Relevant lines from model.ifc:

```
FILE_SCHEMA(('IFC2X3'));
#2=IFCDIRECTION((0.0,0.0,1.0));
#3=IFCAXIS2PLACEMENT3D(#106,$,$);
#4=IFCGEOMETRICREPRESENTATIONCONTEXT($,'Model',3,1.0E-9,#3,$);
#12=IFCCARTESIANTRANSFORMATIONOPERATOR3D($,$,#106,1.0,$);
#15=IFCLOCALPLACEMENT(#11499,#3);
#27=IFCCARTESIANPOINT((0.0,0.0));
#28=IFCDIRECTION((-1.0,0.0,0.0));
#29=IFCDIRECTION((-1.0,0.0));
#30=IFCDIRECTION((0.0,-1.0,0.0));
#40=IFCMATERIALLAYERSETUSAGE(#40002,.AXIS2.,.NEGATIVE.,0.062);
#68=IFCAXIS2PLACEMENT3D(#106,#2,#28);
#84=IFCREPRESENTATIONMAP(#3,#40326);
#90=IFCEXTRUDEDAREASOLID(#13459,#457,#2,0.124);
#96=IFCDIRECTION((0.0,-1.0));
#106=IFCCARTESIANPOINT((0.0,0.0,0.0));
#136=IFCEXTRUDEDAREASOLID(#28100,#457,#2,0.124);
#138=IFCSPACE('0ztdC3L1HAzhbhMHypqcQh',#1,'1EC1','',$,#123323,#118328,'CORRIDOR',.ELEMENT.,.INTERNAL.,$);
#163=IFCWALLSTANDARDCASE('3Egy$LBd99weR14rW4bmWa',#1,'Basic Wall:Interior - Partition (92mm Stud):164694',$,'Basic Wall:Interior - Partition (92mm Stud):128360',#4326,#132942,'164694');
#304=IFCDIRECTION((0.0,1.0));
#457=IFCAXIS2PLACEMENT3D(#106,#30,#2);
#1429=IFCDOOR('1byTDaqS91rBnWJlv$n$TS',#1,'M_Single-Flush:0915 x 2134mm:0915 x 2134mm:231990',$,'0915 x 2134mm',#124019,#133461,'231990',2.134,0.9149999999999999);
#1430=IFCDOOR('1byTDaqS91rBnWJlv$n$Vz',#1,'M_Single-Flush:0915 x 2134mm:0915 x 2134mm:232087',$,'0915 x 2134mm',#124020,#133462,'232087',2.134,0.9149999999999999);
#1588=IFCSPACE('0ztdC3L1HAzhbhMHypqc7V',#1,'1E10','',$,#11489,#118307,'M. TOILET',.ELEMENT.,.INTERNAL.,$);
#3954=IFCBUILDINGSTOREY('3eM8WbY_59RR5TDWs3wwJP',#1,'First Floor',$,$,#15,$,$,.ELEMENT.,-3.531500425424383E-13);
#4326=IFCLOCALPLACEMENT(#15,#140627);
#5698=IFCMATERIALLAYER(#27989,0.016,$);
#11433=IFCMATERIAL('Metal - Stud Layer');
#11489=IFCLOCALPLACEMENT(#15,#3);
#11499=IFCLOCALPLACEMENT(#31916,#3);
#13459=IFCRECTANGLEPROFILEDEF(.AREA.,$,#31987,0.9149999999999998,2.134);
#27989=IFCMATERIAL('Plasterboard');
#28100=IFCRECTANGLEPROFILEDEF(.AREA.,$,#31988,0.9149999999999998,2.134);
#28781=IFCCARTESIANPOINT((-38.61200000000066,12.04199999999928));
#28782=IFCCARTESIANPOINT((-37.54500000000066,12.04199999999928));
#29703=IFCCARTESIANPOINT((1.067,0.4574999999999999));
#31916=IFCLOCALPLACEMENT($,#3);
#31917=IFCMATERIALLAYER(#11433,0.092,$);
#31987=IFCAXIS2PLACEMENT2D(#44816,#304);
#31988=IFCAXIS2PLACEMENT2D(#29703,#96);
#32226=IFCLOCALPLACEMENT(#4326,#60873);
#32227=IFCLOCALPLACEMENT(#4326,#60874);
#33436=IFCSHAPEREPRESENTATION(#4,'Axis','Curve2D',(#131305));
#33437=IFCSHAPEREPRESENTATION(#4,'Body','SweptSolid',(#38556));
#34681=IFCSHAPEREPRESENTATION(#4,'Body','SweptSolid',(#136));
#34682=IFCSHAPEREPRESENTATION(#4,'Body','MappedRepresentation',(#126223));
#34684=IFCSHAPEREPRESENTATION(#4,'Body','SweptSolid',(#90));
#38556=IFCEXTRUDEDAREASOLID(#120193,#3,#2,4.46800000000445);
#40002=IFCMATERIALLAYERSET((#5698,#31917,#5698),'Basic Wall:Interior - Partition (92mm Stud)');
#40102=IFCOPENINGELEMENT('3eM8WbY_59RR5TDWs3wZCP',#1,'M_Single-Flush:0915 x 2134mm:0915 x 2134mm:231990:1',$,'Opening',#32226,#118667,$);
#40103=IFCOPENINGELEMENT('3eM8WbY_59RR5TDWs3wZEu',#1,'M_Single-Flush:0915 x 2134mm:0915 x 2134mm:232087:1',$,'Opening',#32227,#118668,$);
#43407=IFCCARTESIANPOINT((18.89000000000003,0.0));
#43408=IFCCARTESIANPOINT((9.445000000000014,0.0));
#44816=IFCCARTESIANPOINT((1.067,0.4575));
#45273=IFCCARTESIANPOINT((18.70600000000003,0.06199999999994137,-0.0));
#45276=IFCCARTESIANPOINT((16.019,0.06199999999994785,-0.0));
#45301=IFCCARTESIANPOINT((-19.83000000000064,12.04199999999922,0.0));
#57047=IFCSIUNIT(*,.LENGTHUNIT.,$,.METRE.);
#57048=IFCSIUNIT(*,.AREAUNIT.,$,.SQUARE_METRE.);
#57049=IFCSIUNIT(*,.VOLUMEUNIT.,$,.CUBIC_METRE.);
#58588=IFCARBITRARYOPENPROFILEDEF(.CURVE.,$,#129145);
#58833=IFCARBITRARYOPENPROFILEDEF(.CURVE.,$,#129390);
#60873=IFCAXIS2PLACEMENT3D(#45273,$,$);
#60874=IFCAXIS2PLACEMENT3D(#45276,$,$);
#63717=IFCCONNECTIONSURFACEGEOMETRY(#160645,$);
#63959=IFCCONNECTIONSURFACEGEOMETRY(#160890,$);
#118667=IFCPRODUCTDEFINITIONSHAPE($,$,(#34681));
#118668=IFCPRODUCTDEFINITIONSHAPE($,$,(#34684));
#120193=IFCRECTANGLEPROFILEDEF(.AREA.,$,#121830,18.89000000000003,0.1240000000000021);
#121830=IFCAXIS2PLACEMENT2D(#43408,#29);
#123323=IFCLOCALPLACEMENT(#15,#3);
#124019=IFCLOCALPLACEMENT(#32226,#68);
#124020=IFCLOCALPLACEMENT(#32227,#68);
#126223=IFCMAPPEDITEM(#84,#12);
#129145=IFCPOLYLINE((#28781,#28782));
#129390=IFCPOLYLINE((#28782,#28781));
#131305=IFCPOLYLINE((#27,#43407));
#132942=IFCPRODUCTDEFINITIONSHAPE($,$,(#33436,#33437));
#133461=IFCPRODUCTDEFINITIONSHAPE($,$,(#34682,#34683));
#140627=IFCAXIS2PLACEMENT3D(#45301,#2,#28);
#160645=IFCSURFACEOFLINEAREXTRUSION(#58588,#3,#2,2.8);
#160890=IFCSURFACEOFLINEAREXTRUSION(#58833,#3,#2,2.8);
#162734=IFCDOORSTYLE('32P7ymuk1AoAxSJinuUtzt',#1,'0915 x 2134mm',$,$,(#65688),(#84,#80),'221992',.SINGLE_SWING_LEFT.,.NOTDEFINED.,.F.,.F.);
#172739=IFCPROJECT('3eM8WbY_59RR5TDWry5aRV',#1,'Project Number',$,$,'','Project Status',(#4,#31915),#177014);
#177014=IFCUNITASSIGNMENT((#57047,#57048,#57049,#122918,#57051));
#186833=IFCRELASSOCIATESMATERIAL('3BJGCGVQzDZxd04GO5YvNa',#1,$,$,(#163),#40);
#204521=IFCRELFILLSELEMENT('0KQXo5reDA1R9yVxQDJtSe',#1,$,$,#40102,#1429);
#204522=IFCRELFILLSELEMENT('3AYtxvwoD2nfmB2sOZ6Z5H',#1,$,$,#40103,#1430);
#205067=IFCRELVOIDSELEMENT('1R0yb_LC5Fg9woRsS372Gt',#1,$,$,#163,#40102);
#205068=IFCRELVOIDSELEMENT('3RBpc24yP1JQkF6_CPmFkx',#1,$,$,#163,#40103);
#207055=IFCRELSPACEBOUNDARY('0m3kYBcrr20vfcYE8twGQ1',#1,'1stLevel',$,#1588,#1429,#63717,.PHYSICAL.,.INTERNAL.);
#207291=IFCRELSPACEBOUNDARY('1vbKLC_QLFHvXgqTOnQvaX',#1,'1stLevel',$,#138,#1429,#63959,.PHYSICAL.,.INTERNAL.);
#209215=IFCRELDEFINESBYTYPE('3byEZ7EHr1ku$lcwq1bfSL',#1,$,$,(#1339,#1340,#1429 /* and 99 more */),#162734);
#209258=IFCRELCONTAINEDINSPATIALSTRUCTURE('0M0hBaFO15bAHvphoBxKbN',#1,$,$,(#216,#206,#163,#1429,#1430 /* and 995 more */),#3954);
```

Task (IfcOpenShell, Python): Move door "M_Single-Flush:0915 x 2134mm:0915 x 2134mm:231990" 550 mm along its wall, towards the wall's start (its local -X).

```python
import numpy as np
import ifcopenshell
import ifcopenshell.api.geometry
import ifcopenshell.util.placement
import ifcopenshell.util.unit

model = ifcopenshell.open("model.ifc")
unit_scale = ifcopenshell.util.unit.calculate_unit_scale(model)

door = model.by_guid("1byTDaqS91rBnWJlv$n$TS")
opening = door.FillsVoids[0].RelatingOpeningElement
wall = opening.VoidsElements[0].RelatingBuildingElement

wall_matrix = ifcopenshell.util.placement.get_local_placement(wall.ObjectPlacement)
shift = wall_matrix[:3, 0] * -0.55 / unit_scale
before = ifcopenshell.util.placement.get_local_placement(door.ObjectPlacement)[:3, 3].copy()

# The door is placed relative to its opening, so it follows when the opening moves.
matrix = ifcopenshell.util.placement.get_local_placement(opening.ObjectPlacement)
matrix[:3, 3] += shift
ifcopenshell.api.geometry.edit_object_placement(
    model, product=opening, matrix=matrix, is_si=False, should_transform_children=True
)

# Space boundary surfaces are stored in each space's coordinates; move them too.
for rel in door.ProvidesBoundaries:
    if not rel.ConnectionGeometry:
        continue
    surface = rel.ConnectionGeometry.SurfaceOnRelatingElement
    space_matrix = ifcopenshell.util.placement.get_local_placement(rel.RelatingSpace.ObjectPlacement)
    point = np.array(surface.Position.Location.Coordinates) + space_matrix[:3, :3].T @ shift
    surface.Position = model.createIfcAxis2Placement3D(
        model.createIfcCartesianPoint(point.tolist()), surface.Position.Axis, surface.Position.RefDirection
    )

after = ifcopenshell.util.placement.get_local_placement(door.ObjectPlacement)[:3, 3]
print("door moved by", (after - before).round(3) + 0.0)

model.write("model_v2.ifc")
```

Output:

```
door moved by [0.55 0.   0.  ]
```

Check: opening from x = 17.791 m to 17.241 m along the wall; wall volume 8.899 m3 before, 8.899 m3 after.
